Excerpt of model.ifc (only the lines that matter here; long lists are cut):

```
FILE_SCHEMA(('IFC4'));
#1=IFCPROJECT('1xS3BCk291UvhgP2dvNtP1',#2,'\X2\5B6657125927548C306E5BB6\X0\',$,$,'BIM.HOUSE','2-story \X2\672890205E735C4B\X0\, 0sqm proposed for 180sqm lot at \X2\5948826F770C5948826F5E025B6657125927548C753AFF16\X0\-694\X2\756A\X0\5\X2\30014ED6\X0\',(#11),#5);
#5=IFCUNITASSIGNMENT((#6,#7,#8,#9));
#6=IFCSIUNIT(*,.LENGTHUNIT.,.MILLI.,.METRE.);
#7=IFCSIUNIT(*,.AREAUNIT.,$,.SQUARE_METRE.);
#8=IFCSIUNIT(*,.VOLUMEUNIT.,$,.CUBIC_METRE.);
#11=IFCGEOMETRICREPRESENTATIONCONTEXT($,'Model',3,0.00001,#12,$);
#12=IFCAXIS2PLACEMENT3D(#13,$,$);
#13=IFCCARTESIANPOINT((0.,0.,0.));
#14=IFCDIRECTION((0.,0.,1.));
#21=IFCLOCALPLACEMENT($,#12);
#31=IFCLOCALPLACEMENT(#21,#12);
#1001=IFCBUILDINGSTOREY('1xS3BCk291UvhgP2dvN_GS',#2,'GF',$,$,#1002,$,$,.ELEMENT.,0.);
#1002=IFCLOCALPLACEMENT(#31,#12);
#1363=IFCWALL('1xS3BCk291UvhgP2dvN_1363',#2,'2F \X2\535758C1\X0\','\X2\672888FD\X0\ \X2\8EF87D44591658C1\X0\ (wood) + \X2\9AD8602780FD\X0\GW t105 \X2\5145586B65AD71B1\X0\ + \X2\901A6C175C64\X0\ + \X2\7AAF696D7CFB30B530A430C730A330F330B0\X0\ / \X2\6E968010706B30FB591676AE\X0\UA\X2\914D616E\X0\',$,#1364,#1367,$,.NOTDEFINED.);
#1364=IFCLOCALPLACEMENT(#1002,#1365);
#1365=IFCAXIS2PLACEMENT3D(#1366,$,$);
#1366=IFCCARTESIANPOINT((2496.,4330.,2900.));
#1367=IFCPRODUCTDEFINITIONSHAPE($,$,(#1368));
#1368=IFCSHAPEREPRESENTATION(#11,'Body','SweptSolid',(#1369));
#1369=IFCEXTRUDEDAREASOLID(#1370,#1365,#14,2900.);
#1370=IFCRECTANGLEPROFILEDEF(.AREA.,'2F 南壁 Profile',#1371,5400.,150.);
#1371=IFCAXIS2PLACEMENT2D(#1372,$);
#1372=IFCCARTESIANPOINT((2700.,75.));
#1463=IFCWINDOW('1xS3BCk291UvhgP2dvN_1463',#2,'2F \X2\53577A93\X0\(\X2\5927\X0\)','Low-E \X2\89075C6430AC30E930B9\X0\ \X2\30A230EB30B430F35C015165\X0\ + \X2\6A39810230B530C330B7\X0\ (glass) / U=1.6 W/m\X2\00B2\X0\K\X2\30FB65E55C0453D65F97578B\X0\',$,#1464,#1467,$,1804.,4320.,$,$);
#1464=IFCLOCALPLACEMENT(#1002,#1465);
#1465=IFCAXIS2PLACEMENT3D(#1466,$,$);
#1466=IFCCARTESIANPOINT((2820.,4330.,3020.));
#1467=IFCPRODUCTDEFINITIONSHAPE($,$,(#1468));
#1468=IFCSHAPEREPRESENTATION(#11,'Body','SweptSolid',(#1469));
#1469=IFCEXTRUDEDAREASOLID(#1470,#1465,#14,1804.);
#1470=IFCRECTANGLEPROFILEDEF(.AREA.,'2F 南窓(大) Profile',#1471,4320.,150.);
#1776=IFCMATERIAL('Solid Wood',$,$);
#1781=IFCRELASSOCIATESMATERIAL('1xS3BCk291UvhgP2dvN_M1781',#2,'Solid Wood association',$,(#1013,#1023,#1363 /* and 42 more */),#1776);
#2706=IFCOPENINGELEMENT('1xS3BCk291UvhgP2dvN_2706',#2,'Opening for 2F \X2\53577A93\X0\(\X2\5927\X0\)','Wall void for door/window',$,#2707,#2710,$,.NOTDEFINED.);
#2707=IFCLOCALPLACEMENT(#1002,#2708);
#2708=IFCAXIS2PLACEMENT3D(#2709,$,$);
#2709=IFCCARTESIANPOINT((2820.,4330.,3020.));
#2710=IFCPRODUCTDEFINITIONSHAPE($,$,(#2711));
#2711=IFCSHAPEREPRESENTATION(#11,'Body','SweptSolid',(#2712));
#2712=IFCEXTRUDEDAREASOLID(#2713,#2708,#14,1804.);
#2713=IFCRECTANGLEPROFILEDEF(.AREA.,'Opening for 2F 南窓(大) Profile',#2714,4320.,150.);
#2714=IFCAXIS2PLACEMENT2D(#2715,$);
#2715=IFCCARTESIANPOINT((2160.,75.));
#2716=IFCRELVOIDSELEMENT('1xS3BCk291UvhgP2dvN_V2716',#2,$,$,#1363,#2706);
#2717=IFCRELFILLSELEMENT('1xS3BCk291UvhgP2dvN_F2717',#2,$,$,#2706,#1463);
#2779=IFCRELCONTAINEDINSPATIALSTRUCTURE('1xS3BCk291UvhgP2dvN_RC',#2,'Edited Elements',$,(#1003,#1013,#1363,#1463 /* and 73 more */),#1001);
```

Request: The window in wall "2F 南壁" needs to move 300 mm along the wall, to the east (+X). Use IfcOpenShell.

```python
import ifcopenshell
import ifcopenshell.api.geometry
import ifcopenshell.util.placement

model = ifcopenshell.open("model.ifc")

window = model.by_guid("1xS3BCk291UvhgP2dvN_1463")
opening = window.FillsVoids[0].RelatingOpeningElement
wall = opening.VoidsElements[0].RelatingBuildingElement

wall_matrix = ifcopenshell.util.placement.get_local_placement(wall.ObjectPlacement)
shift = wall_matrix[:3, 0] * 300.0
before = ifcopenshell.util.placement.get_local_placement(window.ObjectPlacement)[:3, 3].copy()

# The window is not placed relative to its opening, so move both.
for product in (opening, window):
    matrix = ifcopenshell.util.placement.get_local_placement(product.ObjectPlacement)
    matrix[:3, 3] += shift
    ifcopenshell.api.geometry.edit_object_placement(model, product=product, matrix=matrix, is_si=False)

after = ifcopenshell.util.placement.get_local_placement(window.ObjectPlacement)[:3, 3]
print("window moved by", (after - before).round(3) + 0.0)

model.write("model_updated.ifc")
```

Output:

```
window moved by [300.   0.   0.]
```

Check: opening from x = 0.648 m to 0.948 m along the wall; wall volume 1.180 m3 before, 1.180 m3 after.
